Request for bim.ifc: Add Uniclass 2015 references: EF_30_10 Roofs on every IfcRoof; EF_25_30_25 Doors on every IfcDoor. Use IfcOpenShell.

First a look at what the model holds.

```python
import ifcopenshell

model = ifcopenshell.open("bim.ifc")
print(model.schema)
print("classifications:", [c.Name for c in model.by_type("IfcClassification")])
for ifc_class in ("IfcDoor", "IfcRoof", "IfcStair", "IfcWall", "IfcWindow"):
    print(ifc_class, len(model.by_type(ifc_class)))
```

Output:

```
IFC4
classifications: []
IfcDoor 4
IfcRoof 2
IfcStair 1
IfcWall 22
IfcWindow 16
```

```python
import ifcopenshell
import ifcopenshell.api.classification

model = ifcopenshell.open("bim.ifc")

system = ifcopenshell.api.classification.add_classification(model, classification="Uniclass 2015")

codes = {
    "IfcRoof": ("EF_30_10", "Roofs"),
    "IfcDoor": ("EF_25_30_25", "Doors"),
}
for ifc_class, (code, name) in codes.items():
    products = model.by_type(ifc_class)
    ifcopenshell.api.classification.add_reference(
        model, products=products, classification=system, identification=code, name=name
    )
    print(code, len(products))

model.write("bim_edited.ifc")
```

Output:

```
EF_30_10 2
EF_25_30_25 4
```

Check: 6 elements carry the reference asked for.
